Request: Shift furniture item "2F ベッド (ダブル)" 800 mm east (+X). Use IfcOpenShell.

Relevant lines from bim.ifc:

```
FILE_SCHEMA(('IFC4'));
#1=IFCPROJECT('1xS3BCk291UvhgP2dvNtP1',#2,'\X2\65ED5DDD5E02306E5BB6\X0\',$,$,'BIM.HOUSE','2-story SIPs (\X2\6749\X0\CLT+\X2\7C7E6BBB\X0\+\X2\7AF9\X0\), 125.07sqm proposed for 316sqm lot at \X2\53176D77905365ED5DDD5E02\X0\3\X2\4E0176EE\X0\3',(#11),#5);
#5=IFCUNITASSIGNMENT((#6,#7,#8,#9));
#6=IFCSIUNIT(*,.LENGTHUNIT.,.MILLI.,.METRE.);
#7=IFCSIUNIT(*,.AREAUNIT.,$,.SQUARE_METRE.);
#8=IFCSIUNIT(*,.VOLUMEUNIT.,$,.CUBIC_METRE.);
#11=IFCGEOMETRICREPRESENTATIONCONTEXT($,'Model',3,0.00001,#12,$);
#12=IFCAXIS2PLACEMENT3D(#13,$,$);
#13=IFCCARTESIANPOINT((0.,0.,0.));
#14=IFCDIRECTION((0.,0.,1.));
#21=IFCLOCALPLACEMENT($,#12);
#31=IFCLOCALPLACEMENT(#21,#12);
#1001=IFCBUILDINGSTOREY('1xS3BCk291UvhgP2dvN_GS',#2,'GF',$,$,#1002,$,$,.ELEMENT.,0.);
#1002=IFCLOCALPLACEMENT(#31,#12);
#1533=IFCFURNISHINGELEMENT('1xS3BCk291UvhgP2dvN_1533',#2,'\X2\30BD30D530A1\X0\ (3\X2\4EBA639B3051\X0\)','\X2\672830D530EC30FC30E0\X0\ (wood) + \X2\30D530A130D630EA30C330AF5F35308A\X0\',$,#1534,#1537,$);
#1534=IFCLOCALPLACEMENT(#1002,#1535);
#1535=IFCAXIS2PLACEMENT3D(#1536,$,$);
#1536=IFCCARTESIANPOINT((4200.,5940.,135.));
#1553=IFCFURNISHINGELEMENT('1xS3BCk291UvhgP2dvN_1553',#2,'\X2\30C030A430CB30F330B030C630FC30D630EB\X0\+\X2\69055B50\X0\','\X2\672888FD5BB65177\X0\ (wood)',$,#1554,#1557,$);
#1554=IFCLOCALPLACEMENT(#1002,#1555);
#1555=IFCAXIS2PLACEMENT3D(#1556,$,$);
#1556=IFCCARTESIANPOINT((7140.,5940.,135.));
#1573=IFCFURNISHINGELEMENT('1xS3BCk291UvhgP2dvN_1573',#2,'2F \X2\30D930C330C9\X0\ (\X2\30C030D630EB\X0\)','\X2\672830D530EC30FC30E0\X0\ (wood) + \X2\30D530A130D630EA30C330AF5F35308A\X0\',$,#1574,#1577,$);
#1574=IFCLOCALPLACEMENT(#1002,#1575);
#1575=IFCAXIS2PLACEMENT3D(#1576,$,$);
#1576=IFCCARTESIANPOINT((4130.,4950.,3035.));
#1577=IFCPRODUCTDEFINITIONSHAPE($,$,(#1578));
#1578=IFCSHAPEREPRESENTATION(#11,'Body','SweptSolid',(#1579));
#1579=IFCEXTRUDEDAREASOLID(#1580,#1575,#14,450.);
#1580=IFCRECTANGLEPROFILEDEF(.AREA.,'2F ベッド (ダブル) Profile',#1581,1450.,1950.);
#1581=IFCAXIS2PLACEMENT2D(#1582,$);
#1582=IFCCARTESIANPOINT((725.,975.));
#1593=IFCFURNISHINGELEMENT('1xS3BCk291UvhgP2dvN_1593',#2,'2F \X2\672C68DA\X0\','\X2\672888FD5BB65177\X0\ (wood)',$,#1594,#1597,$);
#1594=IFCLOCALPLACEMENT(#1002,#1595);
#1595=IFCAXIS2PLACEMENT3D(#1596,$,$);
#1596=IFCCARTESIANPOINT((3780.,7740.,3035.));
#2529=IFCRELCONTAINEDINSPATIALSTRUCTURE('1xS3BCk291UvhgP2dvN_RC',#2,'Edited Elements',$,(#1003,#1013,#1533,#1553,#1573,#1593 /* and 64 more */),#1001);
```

```python
import ifcopenshell
import ifcopenshell.api.geometry
import ifcopenshell.util.placement
import ifcopenshell.util.unit

model = ifcopenshell.open("bim.ifc")
unit_scale = ifcopenshell.util.unit.calculate_unit_scale(model)

item = model.by_guid("1xS3BCk291UvhgP2dvN_1573")
matrix = ifcopenshell.util.placement.get_local_placement(item.ObjectPlacement)
matrix[0, 3] += 0.8 / unit_scale
ifcopenshell.api.geometry.edit_object_placement(model, product=item, matrix=matrix, is_si=False)

print(ifcopenshell.util.placement.get_local_placement(item.ObjectPlacement).round(3) + 0.0)

model.write("bim-out.ifc")
```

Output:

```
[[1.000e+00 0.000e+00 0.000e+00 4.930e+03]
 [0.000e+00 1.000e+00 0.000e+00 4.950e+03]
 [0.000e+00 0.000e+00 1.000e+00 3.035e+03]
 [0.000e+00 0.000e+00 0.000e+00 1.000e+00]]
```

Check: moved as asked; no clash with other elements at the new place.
